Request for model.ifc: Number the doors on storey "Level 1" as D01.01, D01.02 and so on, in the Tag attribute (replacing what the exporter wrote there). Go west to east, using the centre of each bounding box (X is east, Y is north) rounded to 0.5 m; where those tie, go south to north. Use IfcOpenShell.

First a look at what the model holds.

```python
import ifcopenshell
import ifcopenshell.util.element
import ifcopenshell.util.placement

model = ifcopenshell.open("model.ifc")
print(model.schema)
storey = next(s for s in model.by_type("IfcBuildingStorey") if s.Name == "Level 1")
doors = [e for e in ifcopenshell.util.element.get_decomposition(storey) if e.is_a("IfcDoor")]
for e in sorted(doors, key=lambda e: e.id()):
    origin = ifcopenshell.util.placement.get_local_placement(e.ObjectPlacement)[:3, 3]
    print(e.id(), e.Tag, e.Name, origin.round(2) + 0.0, sep=" | ")
```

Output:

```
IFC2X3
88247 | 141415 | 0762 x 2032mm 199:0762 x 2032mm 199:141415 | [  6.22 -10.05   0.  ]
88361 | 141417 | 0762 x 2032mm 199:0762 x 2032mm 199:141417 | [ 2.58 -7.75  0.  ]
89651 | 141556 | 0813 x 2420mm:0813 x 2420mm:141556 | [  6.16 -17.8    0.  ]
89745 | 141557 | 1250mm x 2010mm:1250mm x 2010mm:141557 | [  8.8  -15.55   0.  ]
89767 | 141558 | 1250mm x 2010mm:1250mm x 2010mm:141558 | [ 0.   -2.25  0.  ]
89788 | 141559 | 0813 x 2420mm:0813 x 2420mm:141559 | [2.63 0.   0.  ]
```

```python
import ifcopenshell
import ifcopenshell.geom
import ifcopenshell.util.element
import ifcopenshell.util.shape

model = ifcopenshell.open("model.ifc")
settings = ifcopenshell.geom.settings()
settings.set("use-world-coords", True)


def centre(element):
    shape = ifcopenshell.geom.create_shape(settings, element)
    return ifcopenshell.util.shape.get_bbox_centroid(shape.geometry)


storey = next(s for s in model.by_type("IfcBuildingStorey") if s.Name == "Level 1")
doors = [e for e in ifcopenshell.util.element.get_decomposition(storey) if e.is_a("IfcDoor")]

# Insertion points can sit at a corner or the storey origin, so sort by the geometry (in metres).
centres = {e: centre(e) for e in doors}
doors.sort(key=lambda e: (round(centres[e][0] / 0.5), centres[e][1]))

for i, e in enumerate(doors, start=1):
    number = f"D01.{i:02d}"
    e.Tag = number
    print(e.id(), number)

model.write("model_rev.ifc")
```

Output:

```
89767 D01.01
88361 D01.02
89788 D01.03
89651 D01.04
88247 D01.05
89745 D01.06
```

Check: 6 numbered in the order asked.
